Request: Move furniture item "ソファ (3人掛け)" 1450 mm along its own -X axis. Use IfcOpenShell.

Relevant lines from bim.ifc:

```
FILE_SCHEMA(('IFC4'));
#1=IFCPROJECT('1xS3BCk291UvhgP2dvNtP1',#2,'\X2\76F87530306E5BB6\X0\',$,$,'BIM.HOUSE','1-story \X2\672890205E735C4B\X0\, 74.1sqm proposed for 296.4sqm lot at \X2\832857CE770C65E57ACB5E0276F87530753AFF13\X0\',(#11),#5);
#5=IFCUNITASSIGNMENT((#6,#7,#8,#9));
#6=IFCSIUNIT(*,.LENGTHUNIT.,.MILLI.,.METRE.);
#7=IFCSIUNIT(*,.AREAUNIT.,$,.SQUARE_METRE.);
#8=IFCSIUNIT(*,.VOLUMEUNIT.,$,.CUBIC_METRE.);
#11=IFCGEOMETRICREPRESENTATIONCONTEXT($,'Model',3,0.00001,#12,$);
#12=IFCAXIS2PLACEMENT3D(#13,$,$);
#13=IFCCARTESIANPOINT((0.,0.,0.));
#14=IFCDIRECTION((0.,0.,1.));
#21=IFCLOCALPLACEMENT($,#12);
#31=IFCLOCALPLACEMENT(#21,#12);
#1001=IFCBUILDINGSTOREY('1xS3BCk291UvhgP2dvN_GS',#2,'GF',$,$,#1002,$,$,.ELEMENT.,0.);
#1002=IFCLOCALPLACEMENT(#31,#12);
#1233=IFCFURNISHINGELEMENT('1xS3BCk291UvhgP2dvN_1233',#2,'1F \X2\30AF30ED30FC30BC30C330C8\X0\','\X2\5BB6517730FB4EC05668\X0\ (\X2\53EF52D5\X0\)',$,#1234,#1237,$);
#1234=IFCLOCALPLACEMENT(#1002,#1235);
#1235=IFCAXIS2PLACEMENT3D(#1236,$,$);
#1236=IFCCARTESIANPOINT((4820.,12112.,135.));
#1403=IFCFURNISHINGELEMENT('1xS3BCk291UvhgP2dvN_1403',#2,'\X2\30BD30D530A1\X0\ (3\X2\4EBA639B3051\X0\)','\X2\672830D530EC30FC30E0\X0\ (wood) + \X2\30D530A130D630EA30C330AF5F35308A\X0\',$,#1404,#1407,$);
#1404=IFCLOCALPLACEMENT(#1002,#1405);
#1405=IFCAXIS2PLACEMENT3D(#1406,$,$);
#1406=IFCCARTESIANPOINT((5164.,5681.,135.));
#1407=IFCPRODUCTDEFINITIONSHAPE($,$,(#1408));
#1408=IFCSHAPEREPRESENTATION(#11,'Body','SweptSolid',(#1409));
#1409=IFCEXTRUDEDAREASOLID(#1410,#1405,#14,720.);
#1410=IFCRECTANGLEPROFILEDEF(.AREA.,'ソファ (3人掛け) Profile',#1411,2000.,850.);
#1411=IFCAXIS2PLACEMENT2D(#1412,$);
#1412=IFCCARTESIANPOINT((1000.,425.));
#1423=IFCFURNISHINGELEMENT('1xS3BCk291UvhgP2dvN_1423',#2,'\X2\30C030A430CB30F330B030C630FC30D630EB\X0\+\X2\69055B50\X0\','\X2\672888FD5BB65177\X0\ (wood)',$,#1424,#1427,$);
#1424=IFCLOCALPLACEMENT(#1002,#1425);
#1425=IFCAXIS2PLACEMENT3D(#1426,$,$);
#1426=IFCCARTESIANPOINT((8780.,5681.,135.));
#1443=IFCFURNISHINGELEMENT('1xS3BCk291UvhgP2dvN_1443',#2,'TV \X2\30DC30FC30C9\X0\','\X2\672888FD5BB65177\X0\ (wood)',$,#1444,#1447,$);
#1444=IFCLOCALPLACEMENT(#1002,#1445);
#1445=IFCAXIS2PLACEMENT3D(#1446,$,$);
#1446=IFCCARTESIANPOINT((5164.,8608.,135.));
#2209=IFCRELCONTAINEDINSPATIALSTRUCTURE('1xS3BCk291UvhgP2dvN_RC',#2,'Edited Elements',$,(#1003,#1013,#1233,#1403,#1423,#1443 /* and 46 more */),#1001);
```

```python
import ifcopenshell
import ifcopenshell.api.geometry
import ifcopenshell.util.placement

model = ifcopenshell.open("bim.ifc")

item = model.by_guid("1xS3BCk291UvhgP2dvN_1403")
matrix = ifcopenshell.util.placement.get_local_placement(item.ObjectPlacement)
matrix[:3, 3] -= matrix[:3, 0] * 1450.0
ifcopenshell.api.geometry.edit_object_placement(model, product=item, matrix=matrix, is_si=False)

print(ifcopenshell.util.placement.get_local_placement(item.ObjectPlacement).round(3) + 0.0)

model.write("bim_updated.ifc")
```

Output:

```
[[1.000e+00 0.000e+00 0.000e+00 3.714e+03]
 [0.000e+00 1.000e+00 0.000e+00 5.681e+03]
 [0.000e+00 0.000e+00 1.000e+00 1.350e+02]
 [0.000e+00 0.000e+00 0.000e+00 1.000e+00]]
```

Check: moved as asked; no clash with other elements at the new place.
